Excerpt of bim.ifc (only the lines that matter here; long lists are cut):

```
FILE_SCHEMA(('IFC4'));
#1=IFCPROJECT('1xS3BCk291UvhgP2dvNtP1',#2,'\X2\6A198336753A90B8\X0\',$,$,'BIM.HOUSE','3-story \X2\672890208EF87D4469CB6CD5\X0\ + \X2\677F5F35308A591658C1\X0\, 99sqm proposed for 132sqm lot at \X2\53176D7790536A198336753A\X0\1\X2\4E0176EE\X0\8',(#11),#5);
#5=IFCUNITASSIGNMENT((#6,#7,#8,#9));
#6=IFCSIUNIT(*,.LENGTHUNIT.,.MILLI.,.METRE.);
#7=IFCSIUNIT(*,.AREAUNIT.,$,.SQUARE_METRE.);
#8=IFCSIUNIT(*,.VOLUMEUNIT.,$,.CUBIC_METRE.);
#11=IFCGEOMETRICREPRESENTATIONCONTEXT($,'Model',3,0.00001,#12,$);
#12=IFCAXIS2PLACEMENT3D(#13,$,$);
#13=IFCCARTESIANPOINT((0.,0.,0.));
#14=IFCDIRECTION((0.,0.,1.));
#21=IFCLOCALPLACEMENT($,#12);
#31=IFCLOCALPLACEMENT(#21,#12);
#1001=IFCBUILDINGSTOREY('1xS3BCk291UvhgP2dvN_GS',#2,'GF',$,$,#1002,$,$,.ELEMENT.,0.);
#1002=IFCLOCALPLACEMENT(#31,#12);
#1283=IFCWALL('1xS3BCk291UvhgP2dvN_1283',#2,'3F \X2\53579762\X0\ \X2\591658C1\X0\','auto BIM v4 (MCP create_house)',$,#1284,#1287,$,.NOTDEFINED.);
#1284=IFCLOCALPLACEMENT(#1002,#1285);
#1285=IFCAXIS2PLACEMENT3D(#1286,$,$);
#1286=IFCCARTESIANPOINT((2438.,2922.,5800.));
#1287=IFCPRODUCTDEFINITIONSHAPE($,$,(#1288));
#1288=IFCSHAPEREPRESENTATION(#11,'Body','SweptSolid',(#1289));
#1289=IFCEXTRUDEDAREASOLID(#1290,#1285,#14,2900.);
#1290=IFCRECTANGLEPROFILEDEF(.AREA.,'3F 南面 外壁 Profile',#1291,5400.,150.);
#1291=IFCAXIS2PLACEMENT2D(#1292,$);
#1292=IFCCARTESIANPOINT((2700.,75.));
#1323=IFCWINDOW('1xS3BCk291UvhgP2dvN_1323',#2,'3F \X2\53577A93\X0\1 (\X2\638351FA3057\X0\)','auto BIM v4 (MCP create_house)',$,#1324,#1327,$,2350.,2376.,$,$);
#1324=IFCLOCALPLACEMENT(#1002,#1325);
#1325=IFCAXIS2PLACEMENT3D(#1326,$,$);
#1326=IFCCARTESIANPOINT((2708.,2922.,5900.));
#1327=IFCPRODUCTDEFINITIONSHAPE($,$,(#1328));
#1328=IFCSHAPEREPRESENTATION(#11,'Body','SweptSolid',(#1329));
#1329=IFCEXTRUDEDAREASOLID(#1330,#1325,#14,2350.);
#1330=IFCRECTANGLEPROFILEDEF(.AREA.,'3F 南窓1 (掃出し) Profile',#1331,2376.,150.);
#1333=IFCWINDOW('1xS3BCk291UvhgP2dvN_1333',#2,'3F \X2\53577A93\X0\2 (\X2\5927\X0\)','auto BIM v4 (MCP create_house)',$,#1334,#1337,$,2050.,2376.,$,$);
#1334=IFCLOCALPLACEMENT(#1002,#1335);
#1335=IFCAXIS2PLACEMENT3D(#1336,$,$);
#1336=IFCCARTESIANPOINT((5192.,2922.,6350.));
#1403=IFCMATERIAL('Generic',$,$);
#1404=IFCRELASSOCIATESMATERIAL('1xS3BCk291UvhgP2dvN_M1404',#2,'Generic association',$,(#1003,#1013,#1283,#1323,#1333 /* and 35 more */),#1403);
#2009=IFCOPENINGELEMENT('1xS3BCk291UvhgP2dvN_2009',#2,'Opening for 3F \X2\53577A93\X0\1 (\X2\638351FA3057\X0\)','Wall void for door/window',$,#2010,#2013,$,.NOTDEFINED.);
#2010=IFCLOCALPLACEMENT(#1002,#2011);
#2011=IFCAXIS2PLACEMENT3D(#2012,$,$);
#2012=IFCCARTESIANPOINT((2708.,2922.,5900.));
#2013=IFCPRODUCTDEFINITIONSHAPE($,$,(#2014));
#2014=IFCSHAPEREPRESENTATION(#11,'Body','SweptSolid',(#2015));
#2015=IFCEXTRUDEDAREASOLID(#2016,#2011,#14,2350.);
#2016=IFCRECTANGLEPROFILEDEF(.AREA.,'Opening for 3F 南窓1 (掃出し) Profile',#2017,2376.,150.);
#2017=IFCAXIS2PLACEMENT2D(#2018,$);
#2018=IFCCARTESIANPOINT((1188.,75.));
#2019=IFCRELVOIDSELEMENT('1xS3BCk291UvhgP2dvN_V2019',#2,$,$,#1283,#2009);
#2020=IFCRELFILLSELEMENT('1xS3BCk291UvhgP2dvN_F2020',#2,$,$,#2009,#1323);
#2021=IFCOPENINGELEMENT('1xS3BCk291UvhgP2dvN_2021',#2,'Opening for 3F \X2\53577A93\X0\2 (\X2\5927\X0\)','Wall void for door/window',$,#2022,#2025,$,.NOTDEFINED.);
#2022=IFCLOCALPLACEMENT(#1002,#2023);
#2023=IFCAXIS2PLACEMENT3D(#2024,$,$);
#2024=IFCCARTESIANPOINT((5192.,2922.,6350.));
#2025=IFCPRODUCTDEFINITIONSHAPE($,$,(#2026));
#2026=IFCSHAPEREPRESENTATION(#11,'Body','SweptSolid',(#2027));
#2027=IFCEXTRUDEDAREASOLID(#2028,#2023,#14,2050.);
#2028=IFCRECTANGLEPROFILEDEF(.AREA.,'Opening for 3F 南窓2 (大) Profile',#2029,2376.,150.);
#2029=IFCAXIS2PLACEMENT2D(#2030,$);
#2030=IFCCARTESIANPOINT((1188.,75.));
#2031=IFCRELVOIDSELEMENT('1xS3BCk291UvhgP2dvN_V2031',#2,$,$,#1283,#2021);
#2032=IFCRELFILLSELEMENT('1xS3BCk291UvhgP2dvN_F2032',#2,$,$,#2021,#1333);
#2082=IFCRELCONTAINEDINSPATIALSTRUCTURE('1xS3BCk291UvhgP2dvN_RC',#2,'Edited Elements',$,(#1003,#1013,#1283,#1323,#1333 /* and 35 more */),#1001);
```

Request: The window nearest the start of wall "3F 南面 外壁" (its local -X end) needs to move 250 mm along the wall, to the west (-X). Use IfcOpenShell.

```python
import ifcopenshell
import ifcopenshell.api.geometry
import ifcopenshell.util.placement
import ifcopenshell.util.unit

model = ifcopenshell.open("bim.ifc")
unit_scale = ifcopenshell.util.unit.calculate_unit_scale(model)

window = model.by_id(1323)
opening = window.FillsVoids[0].RelatingOpeningElement
wall = opening.VoidsElements[0].RelatingBuildingElement

wall_matrix = ifcopenshell.util.placement.get_local_placement(wall.ObjectPlacement)
shift = wall_matrix[:3, 0] * -0.25 / unit_scale
before = ifcopenshell.util.placement.get_local_placement(window.ObjectPlacement)[:3, 3].copy()

# The window is not placed relative to its opening, so move both.
for product in (opening, window):
    matrix = ifcopenshell.util.placement.get_local_placement(product.ObjectPlacement)
    matrix[:3, 3] += shift
    ifcopenshell.api.geometry.edit_object_placement(model, product=product, matrix=matrix, is_si=False)

after = ifcopenshell.util.placement.get_local_placement(window.ObjectPlacement)[:3, 3]
print("window moved by", (after - before).round(3) + 0.0)

model.write("bim-out.ifc")
```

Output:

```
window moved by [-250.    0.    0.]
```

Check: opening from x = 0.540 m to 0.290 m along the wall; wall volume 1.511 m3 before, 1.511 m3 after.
